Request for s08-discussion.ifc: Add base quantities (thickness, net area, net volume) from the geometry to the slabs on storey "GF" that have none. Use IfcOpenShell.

First a look at what the model holds.

```python
import ifcopenshell
import ifcopenshell.util.element
import ifcopenshell.util.unit

model = ifcopenshell.open("s08-discussion.ifc")
print(model.schema)
for unit_type in ("LENGTHUNIT", "AREAUNIT", "VOLUMEUNIT"):
    print(unit_type, ifcopenshell.util.unit.calculate_unit_scale(model, unit_type))
storey = next(s for s in model.by_type("IfcBuildingStorey") if s.Name == "GF")
slabs = [e for e in ifcopenshell.util.element.get_decomposition(storey) if e.is_a("IfcSlab")]
for e in sorted(slabs, key=lambda e: e.id()):
    print(e.id(), e.is_a(), e.Name, list(ifcopenshell.util.element.get_psets(e, qtos_only=True)), sep=" | ")
```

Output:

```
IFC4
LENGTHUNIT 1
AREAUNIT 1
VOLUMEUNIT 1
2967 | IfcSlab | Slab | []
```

```python
import ifcopenshell
import ifcopenshell.api.pset
import ifcopenshell.geom
import ifcopenshell.util.element
import ifcopenshell.util.shape
import ifcopenshell.util.unit

model = ifcopenshell.open("s08-discussion.ifc")
unit_scale = ifcopenshell.util.unit.calculate_unit_scale(model)
area_scale = ifcopenshell.util.unit.calculate_unit_scale(model, "AREAUNIT")
volume_scale = ifcopenshell.util.unit.calculate_unit_scale(model, "VOLUMEUNIT")
settings = ifcopenshell.geom.settings()

storey = next(s for s in model.by_type("IfcBuildingStorey") if s.Name == "GF")
slabs = [e for e in ifcopenshell.util.element.get_decomposition(storey) if e.is_a("IfcSlab")]

for e in sorted(slabs, key=lambda e: e.id()):
    if ifcopenshell.util.element.get_psets(e, qtos_only=True, should_inherit=False):
        continue
    # Geometry comes back in metres, in the element's own axes.
    shape = ifcopenshell.geom.create_shape(settings, e)
    values = {
        "Width": ifcopenshell.util.shape.get_z(shape.geometry) / unit_scale,
        "NetArea": ifcopenshell.util.shape.get_footprint_area(shape.geometry) / area_scale,
        "NetVolume": ifcopenshell.util.shape.get_volume(shape.geometry) / volume_scale,
    }
    qto = ifcopenshell.api.pset.add_qto(model, product=e, name="Qto_SlabBaseQuantities")
    ifcopenshell.api.pset.edit_qto(model, qto=qto, properties=values)
    print(e.id(), {k: round(v, 3) for k, v in values.items()})

model.write("s08-discussion-out.ifc")
```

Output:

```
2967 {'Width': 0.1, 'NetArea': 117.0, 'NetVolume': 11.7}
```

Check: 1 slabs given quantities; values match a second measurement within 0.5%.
